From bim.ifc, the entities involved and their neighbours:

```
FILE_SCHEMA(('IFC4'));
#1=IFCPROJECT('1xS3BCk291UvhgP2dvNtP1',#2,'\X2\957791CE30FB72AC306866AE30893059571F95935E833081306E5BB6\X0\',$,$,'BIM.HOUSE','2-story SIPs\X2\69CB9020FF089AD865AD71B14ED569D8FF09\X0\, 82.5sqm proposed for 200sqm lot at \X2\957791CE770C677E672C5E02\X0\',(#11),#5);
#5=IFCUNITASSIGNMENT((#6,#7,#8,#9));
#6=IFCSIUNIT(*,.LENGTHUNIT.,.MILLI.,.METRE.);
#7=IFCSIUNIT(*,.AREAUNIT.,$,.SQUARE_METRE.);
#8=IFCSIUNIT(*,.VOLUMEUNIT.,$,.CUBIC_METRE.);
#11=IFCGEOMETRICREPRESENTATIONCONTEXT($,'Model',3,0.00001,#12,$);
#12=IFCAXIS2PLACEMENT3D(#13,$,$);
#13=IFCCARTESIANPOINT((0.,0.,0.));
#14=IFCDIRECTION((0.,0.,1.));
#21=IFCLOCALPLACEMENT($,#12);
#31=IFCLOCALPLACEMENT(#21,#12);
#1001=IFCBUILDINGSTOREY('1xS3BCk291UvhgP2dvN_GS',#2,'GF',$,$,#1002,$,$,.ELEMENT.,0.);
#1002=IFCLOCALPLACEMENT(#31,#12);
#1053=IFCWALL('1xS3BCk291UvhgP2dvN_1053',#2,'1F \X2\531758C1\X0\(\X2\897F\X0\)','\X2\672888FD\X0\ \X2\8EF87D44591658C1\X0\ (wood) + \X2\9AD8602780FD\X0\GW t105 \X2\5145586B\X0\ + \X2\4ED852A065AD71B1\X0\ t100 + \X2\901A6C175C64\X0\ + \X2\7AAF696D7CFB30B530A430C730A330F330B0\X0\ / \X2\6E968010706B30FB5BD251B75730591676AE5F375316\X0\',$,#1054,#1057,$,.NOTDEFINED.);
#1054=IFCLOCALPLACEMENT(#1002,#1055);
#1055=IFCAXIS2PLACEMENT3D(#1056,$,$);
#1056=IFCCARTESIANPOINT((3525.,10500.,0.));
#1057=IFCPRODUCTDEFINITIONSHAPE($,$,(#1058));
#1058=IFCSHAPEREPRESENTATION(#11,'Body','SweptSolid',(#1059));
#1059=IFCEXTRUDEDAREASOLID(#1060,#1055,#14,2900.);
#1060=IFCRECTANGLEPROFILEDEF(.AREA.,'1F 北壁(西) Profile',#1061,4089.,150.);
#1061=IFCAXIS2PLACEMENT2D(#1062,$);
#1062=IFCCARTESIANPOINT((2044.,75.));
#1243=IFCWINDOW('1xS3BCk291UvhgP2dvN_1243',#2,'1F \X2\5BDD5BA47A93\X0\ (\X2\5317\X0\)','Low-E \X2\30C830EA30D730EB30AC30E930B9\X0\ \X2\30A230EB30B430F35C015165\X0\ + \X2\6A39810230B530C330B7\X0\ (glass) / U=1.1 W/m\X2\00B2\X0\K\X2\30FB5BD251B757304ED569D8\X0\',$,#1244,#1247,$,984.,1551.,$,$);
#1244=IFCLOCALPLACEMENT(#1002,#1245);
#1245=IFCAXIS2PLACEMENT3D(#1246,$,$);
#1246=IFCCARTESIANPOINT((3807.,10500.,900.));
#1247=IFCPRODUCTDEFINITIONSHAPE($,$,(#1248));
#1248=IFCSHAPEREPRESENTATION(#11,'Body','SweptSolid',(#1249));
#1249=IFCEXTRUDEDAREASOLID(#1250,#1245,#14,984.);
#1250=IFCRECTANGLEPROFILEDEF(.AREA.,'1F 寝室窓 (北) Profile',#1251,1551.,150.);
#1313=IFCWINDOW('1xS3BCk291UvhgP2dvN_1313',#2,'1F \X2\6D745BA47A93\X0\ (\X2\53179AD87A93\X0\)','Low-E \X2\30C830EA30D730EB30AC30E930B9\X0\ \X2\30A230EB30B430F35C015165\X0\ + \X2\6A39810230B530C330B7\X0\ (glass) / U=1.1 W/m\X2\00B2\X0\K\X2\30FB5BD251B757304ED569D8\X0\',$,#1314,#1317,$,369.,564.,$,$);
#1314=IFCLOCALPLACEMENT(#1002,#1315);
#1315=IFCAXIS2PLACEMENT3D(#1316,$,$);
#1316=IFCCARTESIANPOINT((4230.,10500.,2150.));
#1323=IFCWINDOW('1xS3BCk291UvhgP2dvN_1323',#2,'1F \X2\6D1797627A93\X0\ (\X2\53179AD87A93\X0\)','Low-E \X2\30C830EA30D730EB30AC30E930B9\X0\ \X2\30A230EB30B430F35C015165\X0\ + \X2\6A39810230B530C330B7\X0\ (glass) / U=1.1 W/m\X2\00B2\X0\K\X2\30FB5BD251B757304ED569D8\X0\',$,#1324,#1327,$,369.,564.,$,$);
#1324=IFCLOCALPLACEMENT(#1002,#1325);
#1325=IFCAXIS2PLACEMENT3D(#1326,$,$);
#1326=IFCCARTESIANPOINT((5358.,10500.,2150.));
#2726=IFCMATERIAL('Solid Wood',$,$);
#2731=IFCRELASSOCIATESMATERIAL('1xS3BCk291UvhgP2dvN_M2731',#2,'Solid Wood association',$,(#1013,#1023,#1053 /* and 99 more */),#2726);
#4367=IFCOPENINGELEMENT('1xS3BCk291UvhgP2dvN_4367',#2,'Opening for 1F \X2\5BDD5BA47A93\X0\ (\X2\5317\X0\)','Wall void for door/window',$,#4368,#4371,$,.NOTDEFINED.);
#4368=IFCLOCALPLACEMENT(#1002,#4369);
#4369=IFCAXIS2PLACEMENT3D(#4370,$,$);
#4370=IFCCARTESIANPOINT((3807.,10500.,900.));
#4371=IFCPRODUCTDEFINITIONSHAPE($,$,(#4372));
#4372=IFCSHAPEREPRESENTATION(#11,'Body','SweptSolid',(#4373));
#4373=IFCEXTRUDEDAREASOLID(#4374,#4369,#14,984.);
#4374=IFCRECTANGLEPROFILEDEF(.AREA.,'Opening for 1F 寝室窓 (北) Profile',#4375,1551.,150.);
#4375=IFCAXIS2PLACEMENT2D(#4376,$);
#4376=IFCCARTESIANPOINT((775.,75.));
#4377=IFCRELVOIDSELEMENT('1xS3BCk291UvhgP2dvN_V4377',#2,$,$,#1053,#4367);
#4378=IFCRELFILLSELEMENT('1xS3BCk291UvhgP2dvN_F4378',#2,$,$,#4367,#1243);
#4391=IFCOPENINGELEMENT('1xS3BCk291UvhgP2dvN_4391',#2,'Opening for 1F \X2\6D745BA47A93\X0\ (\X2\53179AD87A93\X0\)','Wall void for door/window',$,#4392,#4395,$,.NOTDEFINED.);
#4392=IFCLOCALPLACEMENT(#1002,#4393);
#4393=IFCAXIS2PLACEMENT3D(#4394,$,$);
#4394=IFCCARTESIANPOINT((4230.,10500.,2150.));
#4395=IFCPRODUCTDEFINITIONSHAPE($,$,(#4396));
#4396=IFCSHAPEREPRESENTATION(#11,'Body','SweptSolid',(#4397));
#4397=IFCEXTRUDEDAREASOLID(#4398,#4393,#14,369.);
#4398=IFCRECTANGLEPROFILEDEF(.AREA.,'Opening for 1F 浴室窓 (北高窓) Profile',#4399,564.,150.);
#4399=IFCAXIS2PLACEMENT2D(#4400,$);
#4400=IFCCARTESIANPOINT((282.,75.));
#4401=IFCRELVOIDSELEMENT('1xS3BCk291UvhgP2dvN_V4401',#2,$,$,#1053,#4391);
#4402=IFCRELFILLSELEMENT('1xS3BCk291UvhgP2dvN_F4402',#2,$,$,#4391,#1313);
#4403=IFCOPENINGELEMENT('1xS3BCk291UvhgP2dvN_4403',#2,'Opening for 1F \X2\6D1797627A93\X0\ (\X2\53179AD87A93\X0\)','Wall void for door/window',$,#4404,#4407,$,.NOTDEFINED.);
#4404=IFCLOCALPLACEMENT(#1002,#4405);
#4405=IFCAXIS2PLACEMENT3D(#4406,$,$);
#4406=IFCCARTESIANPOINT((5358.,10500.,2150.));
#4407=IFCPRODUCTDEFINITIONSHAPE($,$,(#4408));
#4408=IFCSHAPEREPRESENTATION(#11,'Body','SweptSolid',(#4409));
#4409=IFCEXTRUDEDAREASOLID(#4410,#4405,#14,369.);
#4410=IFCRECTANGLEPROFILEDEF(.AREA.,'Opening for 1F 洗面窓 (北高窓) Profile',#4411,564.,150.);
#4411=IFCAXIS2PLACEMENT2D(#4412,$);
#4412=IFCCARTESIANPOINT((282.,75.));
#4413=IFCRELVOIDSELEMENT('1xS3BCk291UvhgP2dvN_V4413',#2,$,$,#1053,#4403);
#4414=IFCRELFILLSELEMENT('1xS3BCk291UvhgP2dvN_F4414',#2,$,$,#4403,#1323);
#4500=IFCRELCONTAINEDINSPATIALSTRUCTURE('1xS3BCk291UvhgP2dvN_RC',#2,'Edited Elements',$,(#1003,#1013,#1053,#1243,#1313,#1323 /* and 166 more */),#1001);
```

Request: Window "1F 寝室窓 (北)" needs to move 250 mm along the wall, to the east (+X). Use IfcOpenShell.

```python
import ifcopenshell
import ifcopenshell.api.geometry
import ifcopenshell.util.placement

model = ifcopenshell.open("bim.ifc")

window = model.by_id(1243)
opening = window.FillsVoids[0].RelatingOpeningElement
wall = opening.VoidsElements[0].RelatingBuildingElement

wall_matrix = ifcopenshell.util.placement.get_local_placement(wall.ObjectPlacement)
shift = wall_matrix[:3, 0] * 250.0
before = ifcopenshell.util.placement.get_local_placement(window.ObjectPlacement)[:3, 3].copy()

# The window is not placed relative to its opening, so move both.
for product in (opening, window):
    matrix = ifcopenshell.util.placement.get_local_placement(product.ObjectPlacement)
    matrix[:3, 3] += shift
    ifcopenshell.api.geometry.edit_object_placement(model, product=product, matrix=matrix, is_si=False)

after = ifcopenshell.util.placement.get_local_placement(window.ObjectPlacement)[:3, 3]
print("window moved by", (after - before).round(3) + 0.0)

model.write("bim_updated.ifc")
```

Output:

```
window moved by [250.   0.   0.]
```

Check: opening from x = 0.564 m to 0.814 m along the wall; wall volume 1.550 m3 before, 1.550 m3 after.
